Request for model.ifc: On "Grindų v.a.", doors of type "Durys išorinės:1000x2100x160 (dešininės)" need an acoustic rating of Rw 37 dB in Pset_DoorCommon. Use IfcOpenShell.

First a look at what the model holds.

```python
import ifcopenshell
import ifcopenshell.util.element

model = ifcopenshell.open("model.ifc")
print(model.schema)
storey = next(s for s in model.by_type("IfcBuildingStorey") if s.Name == "Grindų v.a.")
doors = [e for e in ifcopenshell.util.element.get_decomposition(storey) if e.is_a("IfcDoor")]
seen = {}
for e in doors:
    element_type = ifcopenshell.util.element.get_type(e)
    key = (element_type.Name if element_type != e and element_type else None, ifcopenshell.util.element.get_pset(e, "Pset_DoorCommon", "AcousticRating"))
    seen[key] = seen.get(key, 0) + 1
for (name, value), count in sorted(seen.items(), key=str):
    print(count, "x", name, "|", value)
```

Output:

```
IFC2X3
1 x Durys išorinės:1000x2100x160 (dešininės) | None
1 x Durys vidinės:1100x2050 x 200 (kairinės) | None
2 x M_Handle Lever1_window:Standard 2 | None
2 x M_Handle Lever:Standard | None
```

```python
import ifcopenshell
import ifcopenshell.api.pset
import ifcopenshell.util.element

model = ifcopenshell.open("model.ifc")

storey = next(s for s in model.by_type("IfcBuildingStorey") if s.Name == "Grindų v.a.")
doors = [e for e in ifcopenshell.util.element.get_decomposition(storey) if e.is_a("IfcDoor")]

count = 0
for e in doors:
    element_type = ifcopenshell.util.element.get_type(e)
    if element_type in (None, e) or element_type.Name != "Durys išorinės:1000x2100x160 (dešininės)":
        continue
    # add_pset returns the element's existing set when there is one.
    pset = ifcopenshell.api.pset.add_pset(model, product=e, name="Pset_DoorCommon")
    ifcopenshell.api.pset.edit_pset(model, pset=pset, properties={"AcousticRating": "Rw 37 dB"})
    count += 1

print(count, "doors updated")

model.write("model_updated.ifc")
```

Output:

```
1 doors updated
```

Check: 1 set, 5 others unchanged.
